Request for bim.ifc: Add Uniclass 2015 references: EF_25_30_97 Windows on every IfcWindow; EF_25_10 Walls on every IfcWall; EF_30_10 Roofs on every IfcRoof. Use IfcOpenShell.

First a look at what the model holds.

```python
import ifcopenshell

model = ifcopenshell.open("bim.ifc")
print(model.schema)
print("classifications:", [c.Name for c in model.by_type("IfcClassification")])
for ifc_class in ("IfcDoor", "IfcRoof", "IfcStair", "IfcWall", "IfcWindow"):
    print(ifc_class, len(model.by_type(ifc_class)))
```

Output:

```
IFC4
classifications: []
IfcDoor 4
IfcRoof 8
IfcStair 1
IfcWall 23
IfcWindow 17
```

```python
import ifcopenshell
import ifcopenshell.api.classification

model = ifcopenshell.open("bim.ifc")

system = ifcopenshell.api.classification.add_classification(model, classification="Uniclass 2015")

codes = {
    "IfcWindow": ("EF_25_30_97", "Windows"),
    "IfcWall": ("EF_25_10", "Walls"),
    "IfcRoof": ("EF_30_10", "Roofs"),
}
for ifc_class, (code, name) in codes.items():
    products = model.by_type(ifc_class)
    ifcopenshell.api.classification.add_reference(
        model, products=products, classification=system, identification=code, name=name
    )
    print(code, len(products))

model.write("bim_updated.ifc")
```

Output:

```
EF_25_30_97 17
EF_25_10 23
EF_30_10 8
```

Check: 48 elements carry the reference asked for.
